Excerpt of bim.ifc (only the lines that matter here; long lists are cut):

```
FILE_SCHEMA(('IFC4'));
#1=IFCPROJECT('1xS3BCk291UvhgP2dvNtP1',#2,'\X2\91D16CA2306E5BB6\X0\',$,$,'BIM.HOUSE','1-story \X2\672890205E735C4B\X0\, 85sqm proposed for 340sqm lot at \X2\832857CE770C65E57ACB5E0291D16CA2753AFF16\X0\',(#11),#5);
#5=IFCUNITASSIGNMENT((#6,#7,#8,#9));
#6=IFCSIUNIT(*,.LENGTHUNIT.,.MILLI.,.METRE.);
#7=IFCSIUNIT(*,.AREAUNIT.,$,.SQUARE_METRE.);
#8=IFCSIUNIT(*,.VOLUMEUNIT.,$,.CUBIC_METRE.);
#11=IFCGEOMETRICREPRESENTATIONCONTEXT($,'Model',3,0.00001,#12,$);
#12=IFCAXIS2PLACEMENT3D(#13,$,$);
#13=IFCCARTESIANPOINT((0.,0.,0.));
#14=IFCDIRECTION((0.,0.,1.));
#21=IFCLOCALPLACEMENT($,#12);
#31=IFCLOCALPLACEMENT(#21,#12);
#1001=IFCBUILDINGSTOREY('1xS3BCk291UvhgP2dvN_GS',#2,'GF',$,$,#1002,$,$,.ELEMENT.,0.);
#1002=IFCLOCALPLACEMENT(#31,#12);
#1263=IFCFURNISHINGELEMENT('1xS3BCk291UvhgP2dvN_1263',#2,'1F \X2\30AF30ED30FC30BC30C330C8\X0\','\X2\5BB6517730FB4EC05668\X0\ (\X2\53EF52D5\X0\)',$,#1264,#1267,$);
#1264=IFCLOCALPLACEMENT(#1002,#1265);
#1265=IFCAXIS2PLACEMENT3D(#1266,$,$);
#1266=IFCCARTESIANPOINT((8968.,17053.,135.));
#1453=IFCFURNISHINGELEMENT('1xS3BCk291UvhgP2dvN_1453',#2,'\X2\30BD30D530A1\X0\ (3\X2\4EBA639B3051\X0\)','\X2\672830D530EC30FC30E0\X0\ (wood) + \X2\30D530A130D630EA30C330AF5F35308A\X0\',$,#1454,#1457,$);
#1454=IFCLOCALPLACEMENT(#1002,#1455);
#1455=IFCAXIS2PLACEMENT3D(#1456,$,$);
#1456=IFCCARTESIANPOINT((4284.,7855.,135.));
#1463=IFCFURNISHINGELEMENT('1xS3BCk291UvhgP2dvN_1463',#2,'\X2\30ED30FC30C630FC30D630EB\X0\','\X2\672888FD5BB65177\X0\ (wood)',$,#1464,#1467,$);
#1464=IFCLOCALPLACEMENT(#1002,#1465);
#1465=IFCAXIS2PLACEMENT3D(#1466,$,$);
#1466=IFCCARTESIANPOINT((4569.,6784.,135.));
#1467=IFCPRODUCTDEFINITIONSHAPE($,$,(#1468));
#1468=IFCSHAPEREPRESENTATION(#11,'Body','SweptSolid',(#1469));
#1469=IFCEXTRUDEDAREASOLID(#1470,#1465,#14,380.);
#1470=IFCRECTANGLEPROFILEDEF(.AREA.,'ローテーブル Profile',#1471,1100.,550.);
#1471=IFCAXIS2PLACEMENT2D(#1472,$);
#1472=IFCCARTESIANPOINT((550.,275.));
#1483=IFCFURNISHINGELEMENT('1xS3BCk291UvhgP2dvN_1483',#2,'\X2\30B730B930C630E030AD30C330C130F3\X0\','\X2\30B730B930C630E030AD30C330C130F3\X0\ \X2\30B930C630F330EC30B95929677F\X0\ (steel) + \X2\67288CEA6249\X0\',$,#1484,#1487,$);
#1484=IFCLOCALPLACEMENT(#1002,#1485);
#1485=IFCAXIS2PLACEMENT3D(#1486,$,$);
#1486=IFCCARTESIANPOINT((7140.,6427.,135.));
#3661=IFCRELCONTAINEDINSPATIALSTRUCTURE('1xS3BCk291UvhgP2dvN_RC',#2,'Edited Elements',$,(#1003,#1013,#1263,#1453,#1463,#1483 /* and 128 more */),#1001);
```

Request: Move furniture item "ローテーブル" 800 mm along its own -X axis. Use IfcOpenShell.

```python
import ifcopenshell
import ifcopenshell.api.geometry
import ifcopenshell.util.placement
import ifcopenshell.util.unit

model = ifcopenshell.open("bim.ifc")
unit_scale = ifcopenshell.util.unit.calculate_unit_scale(model)

item = model.by_id(1463)
matrix = ifcopenshell.util.placement.get_local_placement(item.ObjectPlacement)
matrix[:3, 3] -= matrix[:3, 0] * 0.8 / unit_scale
ifcopenshell.api.geometry.edit_object_placement(model, product=item, matrix=matrix, is_si=False)

print(ifcopenshell.util.placement.get_local_placement(item.ObjectPlacement).round(3) + 0.0)

model.write("bim_edited.ifc")
```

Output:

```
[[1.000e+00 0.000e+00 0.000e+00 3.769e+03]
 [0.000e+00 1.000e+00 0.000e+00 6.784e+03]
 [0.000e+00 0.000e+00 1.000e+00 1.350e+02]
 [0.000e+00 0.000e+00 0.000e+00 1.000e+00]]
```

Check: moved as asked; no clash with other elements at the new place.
